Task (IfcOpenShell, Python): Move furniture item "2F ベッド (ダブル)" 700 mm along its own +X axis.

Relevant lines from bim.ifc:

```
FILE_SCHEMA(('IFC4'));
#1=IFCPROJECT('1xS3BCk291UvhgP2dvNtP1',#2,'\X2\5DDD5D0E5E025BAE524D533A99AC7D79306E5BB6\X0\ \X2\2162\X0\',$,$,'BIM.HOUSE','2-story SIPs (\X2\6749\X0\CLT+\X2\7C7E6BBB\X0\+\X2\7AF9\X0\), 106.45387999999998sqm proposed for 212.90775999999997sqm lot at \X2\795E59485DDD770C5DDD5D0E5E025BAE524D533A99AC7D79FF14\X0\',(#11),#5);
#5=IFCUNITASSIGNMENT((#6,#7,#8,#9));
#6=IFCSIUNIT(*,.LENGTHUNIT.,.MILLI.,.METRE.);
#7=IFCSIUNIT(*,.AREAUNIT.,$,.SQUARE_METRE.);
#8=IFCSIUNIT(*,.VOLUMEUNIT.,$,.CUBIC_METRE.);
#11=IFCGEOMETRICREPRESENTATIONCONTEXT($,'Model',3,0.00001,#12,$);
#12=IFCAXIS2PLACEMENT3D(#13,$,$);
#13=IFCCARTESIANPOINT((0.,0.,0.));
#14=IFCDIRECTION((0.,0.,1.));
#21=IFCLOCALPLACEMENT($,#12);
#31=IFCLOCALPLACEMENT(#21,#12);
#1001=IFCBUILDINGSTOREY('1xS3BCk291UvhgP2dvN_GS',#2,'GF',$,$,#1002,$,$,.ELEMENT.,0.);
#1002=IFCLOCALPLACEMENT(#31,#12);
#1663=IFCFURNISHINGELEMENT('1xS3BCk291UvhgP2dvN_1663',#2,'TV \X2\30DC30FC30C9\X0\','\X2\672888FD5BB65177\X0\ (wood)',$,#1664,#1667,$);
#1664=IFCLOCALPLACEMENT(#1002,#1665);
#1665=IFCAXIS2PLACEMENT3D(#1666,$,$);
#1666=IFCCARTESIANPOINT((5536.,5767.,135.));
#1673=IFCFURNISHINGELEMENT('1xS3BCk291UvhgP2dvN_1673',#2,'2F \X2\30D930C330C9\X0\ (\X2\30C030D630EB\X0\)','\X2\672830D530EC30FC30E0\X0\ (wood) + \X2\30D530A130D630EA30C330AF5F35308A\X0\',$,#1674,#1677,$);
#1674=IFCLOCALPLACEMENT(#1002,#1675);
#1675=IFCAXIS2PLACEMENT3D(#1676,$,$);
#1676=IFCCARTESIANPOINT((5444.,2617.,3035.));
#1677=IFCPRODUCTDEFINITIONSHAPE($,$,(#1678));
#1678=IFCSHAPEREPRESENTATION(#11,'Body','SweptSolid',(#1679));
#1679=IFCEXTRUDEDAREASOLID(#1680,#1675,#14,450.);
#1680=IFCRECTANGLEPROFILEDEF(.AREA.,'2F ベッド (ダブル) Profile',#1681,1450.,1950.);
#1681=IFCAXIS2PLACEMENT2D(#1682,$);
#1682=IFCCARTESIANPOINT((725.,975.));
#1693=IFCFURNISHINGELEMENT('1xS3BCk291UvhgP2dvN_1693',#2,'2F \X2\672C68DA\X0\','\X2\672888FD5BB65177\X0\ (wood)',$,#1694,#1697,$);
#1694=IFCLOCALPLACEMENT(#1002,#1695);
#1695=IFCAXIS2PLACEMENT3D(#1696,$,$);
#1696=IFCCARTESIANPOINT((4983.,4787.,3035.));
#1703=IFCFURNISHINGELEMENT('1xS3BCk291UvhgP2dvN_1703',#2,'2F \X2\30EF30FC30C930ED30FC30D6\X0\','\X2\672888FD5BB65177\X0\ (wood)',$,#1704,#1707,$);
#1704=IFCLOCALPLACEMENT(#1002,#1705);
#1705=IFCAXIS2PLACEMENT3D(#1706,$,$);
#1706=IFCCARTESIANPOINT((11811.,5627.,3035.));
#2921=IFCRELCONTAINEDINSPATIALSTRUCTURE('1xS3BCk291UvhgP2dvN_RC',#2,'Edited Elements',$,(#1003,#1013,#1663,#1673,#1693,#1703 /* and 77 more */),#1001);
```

```python
import ifcopenshell
import ifcopenshell.api.geometry
import ifcopenshell.util.placement

model = ifcopenshell.open("bim.ifc")

item = model.by_id(1673)
matrix = ifcopenshell.util.placement.get_local_placement(item.ObjectPlacement)
matrix[:3, 3] += matrix[:3, 0] * 700.0
ifcopenshell.api.geometry.edit_object_placement(model, product=item, matrix=matrix, is_si=False)

print(ifcopenshell.util.placement.get_local_placement(item.ObjectPlacement).round(3) + 0.0)

model.write("bim_updated.ifc")
```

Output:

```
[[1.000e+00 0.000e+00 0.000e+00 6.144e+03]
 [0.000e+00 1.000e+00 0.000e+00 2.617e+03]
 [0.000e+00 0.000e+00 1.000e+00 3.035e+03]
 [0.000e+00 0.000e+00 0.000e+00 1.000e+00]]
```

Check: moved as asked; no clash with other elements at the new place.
